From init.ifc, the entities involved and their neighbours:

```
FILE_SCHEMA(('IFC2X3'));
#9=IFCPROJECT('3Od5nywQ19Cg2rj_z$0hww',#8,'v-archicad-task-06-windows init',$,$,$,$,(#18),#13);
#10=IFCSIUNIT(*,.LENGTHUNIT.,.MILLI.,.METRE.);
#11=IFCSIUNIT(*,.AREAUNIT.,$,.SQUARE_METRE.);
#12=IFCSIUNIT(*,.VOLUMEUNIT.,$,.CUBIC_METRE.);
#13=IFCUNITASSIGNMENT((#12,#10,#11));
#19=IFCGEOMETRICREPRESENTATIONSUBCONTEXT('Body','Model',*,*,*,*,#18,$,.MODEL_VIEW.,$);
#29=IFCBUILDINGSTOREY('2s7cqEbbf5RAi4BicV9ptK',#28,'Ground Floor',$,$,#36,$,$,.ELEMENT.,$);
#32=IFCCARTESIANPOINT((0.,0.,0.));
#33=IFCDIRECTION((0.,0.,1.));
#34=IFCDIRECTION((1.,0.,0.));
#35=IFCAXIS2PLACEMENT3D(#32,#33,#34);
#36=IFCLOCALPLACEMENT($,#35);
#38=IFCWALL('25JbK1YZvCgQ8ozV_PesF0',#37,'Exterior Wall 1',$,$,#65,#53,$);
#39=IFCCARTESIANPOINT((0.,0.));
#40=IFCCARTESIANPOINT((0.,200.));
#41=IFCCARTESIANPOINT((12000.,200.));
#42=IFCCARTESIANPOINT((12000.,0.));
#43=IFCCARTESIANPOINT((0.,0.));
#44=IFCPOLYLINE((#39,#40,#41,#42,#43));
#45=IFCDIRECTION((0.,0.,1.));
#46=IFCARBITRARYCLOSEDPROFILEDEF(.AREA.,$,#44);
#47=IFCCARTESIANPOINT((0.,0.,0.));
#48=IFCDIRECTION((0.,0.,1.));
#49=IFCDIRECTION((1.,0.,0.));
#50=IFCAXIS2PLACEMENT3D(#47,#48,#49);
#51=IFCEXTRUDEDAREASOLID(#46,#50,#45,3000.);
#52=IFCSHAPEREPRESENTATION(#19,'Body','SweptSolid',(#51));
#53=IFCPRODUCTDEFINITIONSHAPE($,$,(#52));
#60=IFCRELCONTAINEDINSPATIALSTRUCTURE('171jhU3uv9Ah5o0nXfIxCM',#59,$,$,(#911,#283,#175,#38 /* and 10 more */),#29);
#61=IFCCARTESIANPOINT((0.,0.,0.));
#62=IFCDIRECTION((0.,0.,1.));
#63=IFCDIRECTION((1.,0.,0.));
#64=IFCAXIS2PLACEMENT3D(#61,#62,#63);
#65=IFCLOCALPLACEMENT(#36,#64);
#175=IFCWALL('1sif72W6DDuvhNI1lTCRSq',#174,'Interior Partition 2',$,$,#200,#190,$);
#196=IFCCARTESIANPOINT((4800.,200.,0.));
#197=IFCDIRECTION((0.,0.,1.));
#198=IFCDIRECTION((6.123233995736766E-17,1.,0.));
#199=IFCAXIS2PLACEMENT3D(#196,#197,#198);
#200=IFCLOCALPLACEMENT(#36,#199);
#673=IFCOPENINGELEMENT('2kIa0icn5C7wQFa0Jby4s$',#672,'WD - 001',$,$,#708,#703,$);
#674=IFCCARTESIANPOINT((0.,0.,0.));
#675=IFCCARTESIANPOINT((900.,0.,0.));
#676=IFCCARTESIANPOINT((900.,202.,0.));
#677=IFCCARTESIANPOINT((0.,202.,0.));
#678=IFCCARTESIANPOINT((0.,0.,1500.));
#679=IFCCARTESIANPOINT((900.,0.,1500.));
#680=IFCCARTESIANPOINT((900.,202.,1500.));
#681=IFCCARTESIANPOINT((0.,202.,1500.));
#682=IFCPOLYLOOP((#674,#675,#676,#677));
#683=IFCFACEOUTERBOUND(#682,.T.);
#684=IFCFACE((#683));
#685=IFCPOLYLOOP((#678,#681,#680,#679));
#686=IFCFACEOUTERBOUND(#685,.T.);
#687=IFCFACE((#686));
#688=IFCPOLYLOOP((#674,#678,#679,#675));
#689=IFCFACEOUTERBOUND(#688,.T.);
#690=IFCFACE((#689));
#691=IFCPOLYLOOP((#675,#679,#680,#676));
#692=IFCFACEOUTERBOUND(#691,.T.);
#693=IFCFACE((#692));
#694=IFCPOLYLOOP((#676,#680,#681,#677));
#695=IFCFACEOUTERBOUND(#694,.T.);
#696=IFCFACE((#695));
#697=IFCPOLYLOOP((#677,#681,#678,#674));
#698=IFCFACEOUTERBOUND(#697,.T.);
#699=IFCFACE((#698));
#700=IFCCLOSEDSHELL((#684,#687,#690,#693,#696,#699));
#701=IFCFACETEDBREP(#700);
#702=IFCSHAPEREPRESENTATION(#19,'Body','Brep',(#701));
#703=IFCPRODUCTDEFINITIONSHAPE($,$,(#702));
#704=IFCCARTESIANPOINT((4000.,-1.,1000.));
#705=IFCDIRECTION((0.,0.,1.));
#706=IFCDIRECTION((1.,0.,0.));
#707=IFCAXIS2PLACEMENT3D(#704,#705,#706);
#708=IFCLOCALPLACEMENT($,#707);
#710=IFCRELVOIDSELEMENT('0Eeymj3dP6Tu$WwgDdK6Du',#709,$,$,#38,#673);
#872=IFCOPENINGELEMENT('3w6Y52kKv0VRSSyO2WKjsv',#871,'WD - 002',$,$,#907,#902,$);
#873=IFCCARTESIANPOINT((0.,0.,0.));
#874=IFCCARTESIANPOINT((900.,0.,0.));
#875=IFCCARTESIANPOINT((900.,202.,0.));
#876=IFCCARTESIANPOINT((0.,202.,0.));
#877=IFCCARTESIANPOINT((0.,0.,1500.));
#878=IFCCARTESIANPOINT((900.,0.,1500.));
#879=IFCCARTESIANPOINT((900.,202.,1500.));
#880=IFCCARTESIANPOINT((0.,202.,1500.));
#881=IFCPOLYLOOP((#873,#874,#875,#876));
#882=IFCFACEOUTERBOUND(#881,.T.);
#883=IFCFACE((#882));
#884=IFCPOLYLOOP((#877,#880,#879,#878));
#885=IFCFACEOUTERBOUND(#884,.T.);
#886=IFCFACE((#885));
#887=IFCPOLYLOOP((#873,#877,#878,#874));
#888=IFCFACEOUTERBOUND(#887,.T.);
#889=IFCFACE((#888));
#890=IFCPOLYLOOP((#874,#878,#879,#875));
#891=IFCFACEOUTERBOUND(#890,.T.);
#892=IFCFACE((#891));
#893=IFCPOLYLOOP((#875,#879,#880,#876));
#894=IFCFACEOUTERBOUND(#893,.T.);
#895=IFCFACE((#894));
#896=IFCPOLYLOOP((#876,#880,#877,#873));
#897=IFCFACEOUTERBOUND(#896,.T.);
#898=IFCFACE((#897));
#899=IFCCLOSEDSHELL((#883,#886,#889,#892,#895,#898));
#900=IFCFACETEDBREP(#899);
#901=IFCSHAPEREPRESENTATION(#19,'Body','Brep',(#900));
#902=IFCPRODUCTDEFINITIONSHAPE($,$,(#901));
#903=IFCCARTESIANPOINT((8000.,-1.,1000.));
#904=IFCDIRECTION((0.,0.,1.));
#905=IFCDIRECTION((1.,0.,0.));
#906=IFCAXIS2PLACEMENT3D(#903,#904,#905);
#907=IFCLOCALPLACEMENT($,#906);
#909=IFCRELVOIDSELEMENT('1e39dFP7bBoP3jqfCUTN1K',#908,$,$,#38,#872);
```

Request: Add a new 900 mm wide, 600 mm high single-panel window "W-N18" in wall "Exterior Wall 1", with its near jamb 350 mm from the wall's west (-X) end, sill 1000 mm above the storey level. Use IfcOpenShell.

```python
import numpy as np
import ifcopenshell
import ifcopenshell.api.feature
import ifcopenshell.api.geometry
import ifcopenshell.api.root
import ifcopenshell.api.spatial
import ifcopenshell.api.type
import ifcopenshell.geom
import ifcopenshell.util.element
import ifcopenshell.util.placement
import ifcopenshell.util.representation
import ifcopenshell.util.shape
import ifcopenshell.util.unit

model = ifcopenshell.open("init.ifc")
unit_scale = ifcopenshell.util.unit.calculate_unit_scale(model)
settings = ifcopenshell.geom.settings()


def volume(element):
    """Net volume in cubic metres, openings subtracted."""
    shape = ifcopenshell.geom.create_shape(settings, element)
    return ifcopenshell.util.shape.get_volume(shape.geometry)


wall = model.by_guid("25JbK1YZvCgQ8ozV_PesF0")
storey = ifcopenshell.util.element.get_container(wall, ifc_class="IfcBuildingStorey")
context = ifcopenshell.util.representation.get_context(model, "Model", "Body", "MODEL_VIEW")
before = volume(wall)

width, height, from_end, sill = 0.9, 0.6, 0.35, 1  # metres

# The wall runs along its own X axis, and the end named is its -X end.
wall_shape = ifcopenshell.geom.create_shape(settings, wall)
x, y, z = ifcopenshell.util.shape.get_vertices(wall_shape.geometry).T
start = x.min() + from_end
face, thickness = float(y.min()), float(y.max() - y.min())
wall_matrix = ifcopenshell.util.placement.get_local_placement(wall.ObjectPlacement)
level = ifcopenshell.util.placement.get_local_placement(storey.ObjectPlacement)[2, 3]


def in_wall(x, y):
    """Placement at x, y metres in the wall's axes, at sill height."""
    matrix = wall_matrix.copy()
    matrix[:, 3] = wall_matrix @ np.array([x / unit_scale, y / unit_scale, 0.0, 1.0])
    matrix[2, 3] = level + sill / unit_scale
    return matrix


# Opening: a box that overshoots both wall faces by 50 mm.
opening = ifcopenshell.api.root.create_entity(model, ifc_class="IfcOpeningElement")
box = ifcopenshell.api.geometry.add_wall_representation(
    model, context=context, length=width, height=height, thickness=thickness + 0.1
)
ifcopenshell.api.geometry.assign_representation(model, product=opening, representation=box)
ifcopenshell.api.geometry.edit_object_placement(model, product=opening, matrix=in_wall(start, face - 0.05), is_si=False)
ifcopenshell.api.feature.add_feature(model, feature=opening, element=wall)

window = ifcopenshell.api.root.create_entity(model, ifc_class="IfcWindow", name="W-N18")
window.OverallWidth, window.OverallHeight = width / unit_scale, height / unit_scale
body = ifcopenshell.api.geometry.add_window_representation(
    model,
    context=context,
    overall_width=window.OverallWidth,
    overall_height=window.OverallHeight,
    partition_type="SINGLE_PANEL",
)
ifcopenshell.api.geometry.assign_representation(model, product=window, representation=body)
ifcopenshell.api.spatial.assign_container(model, products=[window], relating_structure=storey)
fills = ifcopenshell.api.feature.add_filling(model, opening=opening, element=window)
fills.OwnerHistory = window.OwnerHistory  # required in IFC2X3

# IFC2X3 keeps the operation on the window style.
style = ifcopenshell.api.root.create_entity(model, ifc_class="IfcWindowStyle", name="W-N18")
style.OperationType, style.ConstructionType = "SINGLE_PANEL", "NOTDEFINED"
style.ParameterTakesPrecedence = style.Sizeable = False
ifcopenshell.api.type.assign_type(model, related_objects=[window], relating_type=style)

# Centre the window in the wall's thickness.
ifcopenshell.api.geometry.edit_object_placement(model, product=window, matrix=in_wall(start, face), is_si=False)
window_shape = ifcopenshell.geom.create_shape(settings, window)
depth = ifcopenshell.util.shape.get_vertices(window_shape.geometry)[:, 1]
offset = face + thickness / 2 - (depth.min() + depth.max()) / 2
ifcopenshell.api.geometry.edit_object_placement(model, product=window, matrix=in_wall(start, offset), is_si=False)

after = volume(wall)

print(f"wall volume {before:.3f} -> {after:.3f} m3")

model.write("init_edited.ifc")
```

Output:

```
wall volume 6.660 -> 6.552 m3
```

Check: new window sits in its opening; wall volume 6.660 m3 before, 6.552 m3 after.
